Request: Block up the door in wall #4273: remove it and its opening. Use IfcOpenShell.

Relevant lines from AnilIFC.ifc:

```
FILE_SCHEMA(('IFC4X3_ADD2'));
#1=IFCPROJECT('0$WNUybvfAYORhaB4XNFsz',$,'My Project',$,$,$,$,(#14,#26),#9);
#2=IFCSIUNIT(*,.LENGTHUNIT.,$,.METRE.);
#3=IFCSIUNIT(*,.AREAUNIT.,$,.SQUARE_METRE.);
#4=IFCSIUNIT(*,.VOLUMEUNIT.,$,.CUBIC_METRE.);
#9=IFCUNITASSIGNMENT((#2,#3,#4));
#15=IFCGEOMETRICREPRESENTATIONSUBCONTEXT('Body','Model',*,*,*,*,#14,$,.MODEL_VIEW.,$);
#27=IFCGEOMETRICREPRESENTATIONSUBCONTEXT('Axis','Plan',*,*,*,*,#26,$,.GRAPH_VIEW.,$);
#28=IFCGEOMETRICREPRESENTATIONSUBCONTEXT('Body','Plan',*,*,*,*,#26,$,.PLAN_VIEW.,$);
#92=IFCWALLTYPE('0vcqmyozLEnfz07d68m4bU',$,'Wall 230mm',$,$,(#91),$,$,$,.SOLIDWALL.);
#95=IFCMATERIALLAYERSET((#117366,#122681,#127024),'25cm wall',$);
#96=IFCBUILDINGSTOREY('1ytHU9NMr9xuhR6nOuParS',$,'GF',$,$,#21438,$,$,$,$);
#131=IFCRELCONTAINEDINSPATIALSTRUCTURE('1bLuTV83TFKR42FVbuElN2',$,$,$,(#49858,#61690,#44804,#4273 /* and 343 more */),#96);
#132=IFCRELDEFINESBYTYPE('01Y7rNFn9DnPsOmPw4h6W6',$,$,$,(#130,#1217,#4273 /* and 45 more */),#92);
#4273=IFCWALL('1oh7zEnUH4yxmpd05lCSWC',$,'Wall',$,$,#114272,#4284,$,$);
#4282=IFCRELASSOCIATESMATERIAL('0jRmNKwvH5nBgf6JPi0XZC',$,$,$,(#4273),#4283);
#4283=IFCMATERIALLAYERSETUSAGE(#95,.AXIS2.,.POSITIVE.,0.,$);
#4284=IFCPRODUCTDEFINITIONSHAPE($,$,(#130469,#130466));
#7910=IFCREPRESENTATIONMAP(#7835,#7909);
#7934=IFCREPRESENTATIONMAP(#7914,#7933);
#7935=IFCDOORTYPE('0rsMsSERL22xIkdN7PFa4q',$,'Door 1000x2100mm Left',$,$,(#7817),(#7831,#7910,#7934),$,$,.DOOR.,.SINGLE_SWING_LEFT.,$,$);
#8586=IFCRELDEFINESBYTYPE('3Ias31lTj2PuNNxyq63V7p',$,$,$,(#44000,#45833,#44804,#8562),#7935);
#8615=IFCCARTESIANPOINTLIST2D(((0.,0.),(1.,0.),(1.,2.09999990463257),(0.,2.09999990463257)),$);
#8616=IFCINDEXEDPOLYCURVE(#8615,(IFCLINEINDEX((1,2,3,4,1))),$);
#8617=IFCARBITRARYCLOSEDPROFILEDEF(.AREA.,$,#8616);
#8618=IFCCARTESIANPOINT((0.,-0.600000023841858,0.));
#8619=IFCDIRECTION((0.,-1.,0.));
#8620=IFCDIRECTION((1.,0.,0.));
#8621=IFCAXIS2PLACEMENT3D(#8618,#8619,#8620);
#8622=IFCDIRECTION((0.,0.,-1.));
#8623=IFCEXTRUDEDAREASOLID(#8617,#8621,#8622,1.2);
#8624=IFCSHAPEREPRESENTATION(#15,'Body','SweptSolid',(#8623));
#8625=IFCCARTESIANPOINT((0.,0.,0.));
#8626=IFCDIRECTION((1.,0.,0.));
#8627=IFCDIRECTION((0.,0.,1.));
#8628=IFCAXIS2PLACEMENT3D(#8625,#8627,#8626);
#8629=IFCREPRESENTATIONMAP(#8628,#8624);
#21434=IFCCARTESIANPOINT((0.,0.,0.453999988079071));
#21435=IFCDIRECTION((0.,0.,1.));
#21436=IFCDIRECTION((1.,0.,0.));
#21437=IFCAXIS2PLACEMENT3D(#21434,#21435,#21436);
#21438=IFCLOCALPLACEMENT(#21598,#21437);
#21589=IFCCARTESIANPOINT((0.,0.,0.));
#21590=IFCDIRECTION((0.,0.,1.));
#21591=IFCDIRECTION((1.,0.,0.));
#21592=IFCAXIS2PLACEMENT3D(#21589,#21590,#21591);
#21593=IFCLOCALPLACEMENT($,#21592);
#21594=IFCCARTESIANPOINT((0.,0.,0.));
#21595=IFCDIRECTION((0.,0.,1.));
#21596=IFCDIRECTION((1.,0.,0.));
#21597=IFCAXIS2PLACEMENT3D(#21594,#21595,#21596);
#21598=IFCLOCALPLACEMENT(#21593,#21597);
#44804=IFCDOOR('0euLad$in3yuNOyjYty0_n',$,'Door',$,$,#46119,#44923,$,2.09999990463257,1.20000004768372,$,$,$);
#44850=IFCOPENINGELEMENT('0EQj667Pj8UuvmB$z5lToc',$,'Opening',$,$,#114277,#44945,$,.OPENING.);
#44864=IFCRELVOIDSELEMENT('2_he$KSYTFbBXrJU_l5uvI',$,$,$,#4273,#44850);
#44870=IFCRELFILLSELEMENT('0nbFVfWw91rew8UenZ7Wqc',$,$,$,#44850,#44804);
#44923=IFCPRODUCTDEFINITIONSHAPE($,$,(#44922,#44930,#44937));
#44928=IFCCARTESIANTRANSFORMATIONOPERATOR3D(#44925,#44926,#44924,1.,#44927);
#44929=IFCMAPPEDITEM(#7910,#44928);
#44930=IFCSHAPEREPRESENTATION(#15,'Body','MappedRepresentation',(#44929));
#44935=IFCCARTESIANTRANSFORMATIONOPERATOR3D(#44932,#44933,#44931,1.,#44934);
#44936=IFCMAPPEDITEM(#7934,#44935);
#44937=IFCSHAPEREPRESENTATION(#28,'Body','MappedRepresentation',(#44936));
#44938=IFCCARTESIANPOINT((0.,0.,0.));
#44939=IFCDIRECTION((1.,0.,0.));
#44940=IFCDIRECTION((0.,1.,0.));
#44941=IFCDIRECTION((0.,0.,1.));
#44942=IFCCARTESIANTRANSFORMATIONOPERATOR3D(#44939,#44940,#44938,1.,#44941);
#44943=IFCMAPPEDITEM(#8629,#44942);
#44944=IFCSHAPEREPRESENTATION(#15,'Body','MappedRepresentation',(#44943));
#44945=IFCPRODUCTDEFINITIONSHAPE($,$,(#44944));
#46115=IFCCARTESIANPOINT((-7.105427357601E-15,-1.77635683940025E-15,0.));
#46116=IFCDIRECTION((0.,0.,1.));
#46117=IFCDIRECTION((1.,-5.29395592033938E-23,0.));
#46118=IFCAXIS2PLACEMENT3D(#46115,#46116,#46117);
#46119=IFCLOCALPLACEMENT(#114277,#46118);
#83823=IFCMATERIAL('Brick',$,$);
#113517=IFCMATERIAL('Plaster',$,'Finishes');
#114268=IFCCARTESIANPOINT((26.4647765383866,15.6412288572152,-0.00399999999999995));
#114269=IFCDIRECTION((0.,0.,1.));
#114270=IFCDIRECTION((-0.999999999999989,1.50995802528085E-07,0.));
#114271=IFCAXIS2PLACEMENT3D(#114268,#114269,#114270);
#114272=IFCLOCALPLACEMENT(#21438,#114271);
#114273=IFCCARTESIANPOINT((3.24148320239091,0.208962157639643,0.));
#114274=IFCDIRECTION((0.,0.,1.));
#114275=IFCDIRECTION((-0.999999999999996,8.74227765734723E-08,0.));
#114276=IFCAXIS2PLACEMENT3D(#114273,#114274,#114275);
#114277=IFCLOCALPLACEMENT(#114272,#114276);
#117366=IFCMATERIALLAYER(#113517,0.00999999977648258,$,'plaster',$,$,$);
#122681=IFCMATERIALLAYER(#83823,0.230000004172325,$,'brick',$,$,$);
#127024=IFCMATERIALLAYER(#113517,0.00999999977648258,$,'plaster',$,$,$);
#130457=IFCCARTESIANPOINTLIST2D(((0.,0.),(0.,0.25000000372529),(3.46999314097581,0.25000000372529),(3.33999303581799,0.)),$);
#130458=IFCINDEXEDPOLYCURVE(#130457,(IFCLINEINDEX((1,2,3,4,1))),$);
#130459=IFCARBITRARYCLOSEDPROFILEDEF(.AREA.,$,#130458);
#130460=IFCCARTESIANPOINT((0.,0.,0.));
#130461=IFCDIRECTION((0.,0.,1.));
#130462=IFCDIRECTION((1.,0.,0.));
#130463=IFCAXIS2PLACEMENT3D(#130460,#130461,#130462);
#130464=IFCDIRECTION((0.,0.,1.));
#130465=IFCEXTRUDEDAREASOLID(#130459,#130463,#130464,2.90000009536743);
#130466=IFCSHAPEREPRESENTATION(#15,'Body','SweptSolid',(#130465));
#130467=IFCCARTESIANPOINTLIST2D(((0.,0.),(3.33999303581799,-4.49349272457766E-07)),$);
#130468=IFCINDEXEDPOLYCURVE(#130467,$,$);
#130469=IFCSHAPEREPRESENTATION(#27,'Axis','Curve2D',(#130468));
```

```python
import ifcopenshell
import ifcopenshell.api.feature
import ifcopenshell.api.root
import ifcopenshell.geom
import ifcopenshell.util.shape

model = ifcopenshell.open("AnilIFC.ifc")
settings = ifcopenshell.geom.settings()


def volume(element):
    """Net volume in cubic metres, openings subtracted."""
    shape = ifcopenshell.geom.create_shape(settings, element)
    return ifcopenshell.util.shape.get_volume(shape.geometry)


door = model.by_id(44804)
opening = door.FillsVoids[0].RelatingOpeningElement
wall = opening.VoidsElements[0].RelatingBuildingElement
before = volume(wall)

ifcopenshell.api.root.remove_product(model, product=door)
ifcopenshell.api.feature.remove_feature(model, feature=opening)

after = volume(wall)

print(f"wall volume {before:.3f} -> {after:.3f} m3")

model.write("AnilIFC_edited.ifc")
```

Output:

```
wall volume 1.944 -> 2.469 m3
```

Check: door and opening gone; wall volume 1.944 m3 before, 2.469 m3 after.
